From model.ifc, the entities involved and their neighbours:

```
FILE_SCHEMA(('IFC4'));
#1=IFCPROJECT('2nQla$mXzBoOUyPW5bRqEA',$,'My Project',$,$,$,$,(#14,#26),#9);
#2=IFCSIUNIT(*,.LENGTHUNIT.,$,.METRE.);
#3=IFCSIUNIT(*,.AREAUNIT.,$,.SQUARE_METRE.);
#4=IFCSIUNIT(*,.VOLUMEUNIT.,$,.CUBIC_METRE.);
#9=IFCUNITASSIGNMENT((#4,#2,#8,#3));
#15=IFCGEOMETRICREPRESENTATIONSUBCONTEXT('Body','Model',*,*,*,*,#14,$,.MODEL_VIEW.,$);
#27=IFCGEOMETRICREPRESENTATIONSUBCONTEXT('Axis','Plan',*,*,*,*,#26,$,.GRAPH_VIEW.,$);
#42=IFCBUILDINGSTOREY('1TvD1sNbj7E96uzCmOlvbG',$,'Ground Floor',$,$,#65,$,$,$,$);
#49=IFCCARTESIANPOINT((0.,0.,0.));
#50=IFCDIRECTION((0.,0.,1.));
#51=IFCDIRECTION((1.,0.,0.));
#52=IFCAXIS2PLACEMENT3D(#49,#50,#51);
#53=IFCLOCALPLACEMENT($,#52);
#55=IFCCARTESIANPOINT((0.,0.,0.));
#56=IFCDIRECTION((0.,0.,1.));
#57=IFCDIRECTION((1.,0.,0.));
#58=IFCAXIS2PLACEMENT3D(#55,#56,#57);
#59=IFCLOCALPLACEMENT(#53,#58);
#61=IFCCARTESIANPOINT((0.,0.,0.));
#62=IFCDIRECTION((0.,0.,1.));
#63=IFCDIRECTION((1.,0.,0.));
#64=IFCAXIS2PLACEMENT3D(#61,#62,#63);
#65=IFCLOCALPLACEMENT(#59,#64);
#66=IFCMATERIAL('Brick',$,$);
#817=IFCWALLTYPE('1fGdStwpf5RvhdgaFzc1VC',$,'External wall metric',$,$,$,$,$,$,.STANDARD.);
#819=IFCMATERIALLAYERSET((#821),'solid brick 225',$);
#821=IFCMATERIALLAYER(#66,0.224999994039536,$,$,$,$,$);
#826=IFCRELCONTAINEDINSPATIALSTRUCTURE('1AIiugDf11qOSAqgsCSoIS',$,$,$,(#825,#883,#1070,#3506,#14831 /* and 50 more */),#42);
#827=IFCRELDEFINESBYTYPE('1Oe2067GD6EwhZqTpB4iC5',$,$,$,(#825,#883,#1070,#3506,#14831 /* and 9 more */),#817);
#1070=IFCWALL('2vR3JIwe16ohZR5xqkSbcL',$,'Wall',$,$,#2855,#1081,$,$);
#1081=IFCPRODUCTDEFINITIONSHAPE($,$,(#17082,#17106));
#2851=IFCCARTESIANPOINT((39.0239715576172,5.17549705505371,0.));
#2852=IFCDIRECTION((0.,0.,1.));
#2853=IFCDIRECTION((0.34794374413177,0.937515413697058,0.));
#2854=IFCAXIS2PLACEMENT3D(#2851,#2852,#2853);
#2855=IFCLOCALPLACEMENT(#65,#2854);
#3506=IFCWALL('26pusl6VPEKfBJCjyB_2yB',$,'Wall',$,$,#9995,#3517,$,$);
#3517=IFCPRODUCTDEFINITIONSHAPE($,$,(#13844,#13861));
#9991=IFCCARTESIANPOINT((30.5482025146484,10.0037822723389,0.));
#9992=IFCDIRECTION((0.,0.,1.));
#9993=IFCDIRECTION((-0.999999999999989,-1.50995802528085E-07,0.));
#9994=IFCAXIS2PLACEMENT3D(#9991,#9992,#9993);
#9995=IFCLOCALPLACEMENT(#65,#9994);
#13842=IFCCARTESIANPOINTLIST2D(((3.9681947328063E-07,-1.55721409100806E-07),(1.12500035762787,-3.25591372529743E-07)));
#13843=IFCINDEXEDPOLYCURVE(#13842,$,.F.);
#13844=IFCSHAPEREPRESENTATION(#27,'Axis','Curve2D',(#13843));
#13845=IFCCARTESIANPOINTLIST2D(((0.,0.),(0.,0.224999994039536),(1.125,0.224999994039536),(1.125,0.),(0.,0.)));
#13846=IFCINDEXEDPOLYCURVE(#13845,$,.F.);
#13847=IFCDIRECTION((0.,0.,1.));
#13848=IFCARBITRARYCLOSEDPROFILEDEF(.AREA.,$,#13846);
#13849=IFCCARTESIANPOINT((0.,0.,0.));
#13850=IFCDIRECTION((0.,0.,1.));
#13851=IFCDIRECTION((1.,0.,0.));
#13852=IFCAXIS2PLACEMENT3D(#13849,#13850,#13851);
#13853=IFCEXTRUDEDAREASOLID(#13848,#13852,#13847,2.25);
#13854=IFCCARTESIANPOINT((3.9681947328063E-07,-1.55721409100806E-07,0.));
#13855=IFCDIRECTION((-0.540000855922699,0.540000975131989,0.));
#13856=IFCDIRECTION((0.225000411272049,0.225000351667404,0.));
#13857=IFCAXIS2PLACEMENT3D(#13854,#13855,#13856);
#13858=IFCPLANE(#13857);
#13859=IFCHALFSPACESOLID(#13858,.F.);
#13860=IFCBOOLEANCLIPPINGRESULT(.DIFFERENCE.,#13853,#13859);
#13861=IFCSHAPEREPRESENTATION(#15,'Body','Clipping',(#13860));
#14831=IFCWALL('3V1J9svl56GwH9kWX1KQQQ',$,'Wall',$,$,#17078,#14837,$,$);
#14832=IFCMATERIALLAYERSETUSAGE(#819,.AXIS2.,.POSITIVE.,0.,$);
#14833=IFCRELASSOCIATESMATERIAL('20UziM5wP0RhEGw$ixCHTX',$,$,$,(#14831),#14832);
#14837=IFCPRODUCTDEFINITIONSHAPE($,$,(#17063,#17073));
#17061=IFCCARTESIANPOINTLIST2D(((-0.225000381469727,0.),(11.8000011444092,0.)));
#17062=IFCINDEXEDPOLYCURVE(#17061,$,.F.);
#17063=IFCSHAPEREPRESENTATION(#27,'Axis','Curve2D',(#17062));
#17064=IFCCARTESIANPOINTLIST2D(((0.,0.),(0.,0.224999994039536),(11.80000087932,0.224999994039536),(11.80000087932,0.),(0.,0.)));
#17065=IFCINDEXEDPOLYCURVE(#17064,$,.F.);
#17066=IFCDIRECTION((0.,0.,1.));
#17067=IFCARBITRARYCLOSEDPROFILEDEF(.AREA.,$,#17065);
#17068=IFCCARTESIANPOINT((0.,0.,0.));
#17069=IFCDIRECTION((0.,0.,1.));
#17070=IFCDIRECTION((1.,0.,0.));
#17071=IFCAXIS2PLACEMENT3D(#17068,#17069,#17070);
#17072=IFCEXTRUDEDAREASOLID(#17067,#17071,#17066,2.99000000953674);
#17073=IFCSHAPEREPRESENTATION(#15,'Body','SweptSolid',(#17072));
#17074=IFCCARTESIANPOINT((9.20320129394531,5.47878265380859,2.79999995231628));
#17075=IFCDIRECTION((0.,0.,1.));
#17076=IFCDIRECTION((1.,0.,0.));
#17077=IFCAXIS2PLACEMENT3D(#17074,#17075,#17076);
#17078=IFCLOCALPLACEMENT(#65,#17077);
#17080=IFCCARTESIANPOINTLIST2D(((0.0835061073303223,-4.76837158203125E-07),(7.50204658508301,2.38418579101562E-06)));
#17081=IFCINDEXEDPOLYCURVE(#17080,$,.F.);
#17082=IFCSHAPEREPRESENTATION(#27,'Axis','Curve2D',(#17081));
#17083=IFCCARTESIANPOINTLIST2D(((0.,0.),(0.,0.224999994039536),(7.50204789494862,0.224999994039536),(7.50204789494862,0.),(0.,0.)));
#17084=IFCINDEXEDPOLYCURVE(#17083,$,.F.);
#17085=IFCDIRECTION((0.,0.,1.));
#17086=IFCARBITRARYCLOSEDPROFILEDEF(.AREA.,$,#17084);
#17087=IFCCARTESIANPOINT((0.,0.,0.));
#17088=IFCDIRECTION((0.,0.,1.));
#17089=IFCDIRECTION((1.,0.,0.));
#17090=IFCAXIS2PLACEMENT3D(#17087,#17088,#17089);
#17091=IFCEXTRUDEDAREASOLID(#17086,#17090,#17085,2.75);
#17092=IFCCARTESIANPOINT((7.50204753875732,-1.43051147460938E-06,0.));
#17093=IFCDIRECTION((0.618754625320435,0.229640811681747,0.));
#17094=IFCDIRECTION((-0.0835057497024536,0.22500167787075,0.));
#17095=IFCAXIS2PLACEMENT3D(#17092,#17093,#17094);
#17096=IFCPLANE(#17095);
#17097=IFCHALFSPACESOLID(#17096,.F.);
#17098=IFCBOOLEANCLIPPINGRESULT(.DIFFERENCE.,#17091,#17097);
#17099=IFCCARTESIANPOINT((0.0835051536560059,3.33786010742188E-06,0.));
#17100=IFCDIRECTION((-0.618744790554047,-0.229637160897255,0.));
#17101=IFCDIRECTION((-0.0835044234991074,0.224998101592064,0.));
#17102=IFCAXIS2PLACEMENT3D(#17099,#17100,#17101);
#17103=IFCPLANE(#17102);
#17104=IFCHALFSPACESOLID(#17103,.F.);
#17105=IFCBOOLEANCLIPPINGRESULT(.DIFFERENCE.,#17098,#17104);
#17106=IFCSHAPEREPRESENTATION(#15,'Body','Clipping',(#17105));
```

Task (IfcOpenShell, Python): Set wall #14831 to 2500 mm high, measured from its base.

```python
import ifcopenshell
import ifcopenshell.geom
import ifcopenshell.util.representation
import ifcopenshell.util.shape

model = ifcopenshell.open("model.ifc")
settings = ifcopenshell.geom.settings()


def volume(element):
    """Net volume in cubic metres, openings subtracted."""
    shape = ifcopenshell.geom.create_shape(settings, element)
    return ifcopenshell.util.shape.get_volume(shape.geometry)


wall = model.by_id(14831)
before = volume(wall)

body = ifcopenshell.util.representation.get_representation(wall, "Model", "Body")
solid = body.Items[0]
old_height = solid.Depth
solid.Depth = 2.5
after = volume(wall)

print(f"height {old_height:g} -> {solid.Depth:g}, volume {before:.3f} -> {after:.3f} m3")

model.write("model-out.ifc")
```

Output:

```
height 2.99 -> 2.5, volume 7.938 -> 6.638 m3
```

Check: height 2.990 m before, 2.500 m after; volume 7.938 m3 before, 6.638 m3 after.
